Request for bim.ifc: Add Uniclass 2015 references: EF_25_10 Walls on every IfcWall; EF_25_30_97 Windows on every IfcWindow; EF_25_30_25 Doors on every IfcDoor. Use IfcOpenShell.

First a look at what the model holds.

```python
import ifcopenshell

model = ifcopenshell.open("bim.ifc")
print(model.schema)
print("classifications:", [c.Name for c in model.by_type("IfcClassification")])
for ifc_class in ("IfcDoor", "IfcRoof", "IfcStair", "IfcWall", "IfcWindow"):
    print(ifc_class, len(model.by_type(ifc_class)))
```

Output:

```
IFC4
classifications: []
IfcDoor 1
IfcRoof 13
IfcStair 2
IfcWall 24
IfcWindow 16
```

```python
import ifcopenshell
import ifcopenshell.api.classification

model = ifcopenshell.open("bim.ifc")

system = ifcopenshell.api.classification.add_classification(model, classification="Uniclass 2015")

codes = {
    "IfcWall": ("EF_25_10", "Walls"),
    "IfcWindow": ("EF_25_30_97", "Windows"),
    "IfcDoor": ("EF_25_30_25", "Doors"),
}
for ifc_class, (code, name) in codes.items():
    products = model.by_type(ifc_class)
    ifcopenshell.api.classification.add_reference(
        model, products=products, classification=system, identification=code, name=name
    )
    print(code, len(products))

model.write("bim_rev.ifc")
```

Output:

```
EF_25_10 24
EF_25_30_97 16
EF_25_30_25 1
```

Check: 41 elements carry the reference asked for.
